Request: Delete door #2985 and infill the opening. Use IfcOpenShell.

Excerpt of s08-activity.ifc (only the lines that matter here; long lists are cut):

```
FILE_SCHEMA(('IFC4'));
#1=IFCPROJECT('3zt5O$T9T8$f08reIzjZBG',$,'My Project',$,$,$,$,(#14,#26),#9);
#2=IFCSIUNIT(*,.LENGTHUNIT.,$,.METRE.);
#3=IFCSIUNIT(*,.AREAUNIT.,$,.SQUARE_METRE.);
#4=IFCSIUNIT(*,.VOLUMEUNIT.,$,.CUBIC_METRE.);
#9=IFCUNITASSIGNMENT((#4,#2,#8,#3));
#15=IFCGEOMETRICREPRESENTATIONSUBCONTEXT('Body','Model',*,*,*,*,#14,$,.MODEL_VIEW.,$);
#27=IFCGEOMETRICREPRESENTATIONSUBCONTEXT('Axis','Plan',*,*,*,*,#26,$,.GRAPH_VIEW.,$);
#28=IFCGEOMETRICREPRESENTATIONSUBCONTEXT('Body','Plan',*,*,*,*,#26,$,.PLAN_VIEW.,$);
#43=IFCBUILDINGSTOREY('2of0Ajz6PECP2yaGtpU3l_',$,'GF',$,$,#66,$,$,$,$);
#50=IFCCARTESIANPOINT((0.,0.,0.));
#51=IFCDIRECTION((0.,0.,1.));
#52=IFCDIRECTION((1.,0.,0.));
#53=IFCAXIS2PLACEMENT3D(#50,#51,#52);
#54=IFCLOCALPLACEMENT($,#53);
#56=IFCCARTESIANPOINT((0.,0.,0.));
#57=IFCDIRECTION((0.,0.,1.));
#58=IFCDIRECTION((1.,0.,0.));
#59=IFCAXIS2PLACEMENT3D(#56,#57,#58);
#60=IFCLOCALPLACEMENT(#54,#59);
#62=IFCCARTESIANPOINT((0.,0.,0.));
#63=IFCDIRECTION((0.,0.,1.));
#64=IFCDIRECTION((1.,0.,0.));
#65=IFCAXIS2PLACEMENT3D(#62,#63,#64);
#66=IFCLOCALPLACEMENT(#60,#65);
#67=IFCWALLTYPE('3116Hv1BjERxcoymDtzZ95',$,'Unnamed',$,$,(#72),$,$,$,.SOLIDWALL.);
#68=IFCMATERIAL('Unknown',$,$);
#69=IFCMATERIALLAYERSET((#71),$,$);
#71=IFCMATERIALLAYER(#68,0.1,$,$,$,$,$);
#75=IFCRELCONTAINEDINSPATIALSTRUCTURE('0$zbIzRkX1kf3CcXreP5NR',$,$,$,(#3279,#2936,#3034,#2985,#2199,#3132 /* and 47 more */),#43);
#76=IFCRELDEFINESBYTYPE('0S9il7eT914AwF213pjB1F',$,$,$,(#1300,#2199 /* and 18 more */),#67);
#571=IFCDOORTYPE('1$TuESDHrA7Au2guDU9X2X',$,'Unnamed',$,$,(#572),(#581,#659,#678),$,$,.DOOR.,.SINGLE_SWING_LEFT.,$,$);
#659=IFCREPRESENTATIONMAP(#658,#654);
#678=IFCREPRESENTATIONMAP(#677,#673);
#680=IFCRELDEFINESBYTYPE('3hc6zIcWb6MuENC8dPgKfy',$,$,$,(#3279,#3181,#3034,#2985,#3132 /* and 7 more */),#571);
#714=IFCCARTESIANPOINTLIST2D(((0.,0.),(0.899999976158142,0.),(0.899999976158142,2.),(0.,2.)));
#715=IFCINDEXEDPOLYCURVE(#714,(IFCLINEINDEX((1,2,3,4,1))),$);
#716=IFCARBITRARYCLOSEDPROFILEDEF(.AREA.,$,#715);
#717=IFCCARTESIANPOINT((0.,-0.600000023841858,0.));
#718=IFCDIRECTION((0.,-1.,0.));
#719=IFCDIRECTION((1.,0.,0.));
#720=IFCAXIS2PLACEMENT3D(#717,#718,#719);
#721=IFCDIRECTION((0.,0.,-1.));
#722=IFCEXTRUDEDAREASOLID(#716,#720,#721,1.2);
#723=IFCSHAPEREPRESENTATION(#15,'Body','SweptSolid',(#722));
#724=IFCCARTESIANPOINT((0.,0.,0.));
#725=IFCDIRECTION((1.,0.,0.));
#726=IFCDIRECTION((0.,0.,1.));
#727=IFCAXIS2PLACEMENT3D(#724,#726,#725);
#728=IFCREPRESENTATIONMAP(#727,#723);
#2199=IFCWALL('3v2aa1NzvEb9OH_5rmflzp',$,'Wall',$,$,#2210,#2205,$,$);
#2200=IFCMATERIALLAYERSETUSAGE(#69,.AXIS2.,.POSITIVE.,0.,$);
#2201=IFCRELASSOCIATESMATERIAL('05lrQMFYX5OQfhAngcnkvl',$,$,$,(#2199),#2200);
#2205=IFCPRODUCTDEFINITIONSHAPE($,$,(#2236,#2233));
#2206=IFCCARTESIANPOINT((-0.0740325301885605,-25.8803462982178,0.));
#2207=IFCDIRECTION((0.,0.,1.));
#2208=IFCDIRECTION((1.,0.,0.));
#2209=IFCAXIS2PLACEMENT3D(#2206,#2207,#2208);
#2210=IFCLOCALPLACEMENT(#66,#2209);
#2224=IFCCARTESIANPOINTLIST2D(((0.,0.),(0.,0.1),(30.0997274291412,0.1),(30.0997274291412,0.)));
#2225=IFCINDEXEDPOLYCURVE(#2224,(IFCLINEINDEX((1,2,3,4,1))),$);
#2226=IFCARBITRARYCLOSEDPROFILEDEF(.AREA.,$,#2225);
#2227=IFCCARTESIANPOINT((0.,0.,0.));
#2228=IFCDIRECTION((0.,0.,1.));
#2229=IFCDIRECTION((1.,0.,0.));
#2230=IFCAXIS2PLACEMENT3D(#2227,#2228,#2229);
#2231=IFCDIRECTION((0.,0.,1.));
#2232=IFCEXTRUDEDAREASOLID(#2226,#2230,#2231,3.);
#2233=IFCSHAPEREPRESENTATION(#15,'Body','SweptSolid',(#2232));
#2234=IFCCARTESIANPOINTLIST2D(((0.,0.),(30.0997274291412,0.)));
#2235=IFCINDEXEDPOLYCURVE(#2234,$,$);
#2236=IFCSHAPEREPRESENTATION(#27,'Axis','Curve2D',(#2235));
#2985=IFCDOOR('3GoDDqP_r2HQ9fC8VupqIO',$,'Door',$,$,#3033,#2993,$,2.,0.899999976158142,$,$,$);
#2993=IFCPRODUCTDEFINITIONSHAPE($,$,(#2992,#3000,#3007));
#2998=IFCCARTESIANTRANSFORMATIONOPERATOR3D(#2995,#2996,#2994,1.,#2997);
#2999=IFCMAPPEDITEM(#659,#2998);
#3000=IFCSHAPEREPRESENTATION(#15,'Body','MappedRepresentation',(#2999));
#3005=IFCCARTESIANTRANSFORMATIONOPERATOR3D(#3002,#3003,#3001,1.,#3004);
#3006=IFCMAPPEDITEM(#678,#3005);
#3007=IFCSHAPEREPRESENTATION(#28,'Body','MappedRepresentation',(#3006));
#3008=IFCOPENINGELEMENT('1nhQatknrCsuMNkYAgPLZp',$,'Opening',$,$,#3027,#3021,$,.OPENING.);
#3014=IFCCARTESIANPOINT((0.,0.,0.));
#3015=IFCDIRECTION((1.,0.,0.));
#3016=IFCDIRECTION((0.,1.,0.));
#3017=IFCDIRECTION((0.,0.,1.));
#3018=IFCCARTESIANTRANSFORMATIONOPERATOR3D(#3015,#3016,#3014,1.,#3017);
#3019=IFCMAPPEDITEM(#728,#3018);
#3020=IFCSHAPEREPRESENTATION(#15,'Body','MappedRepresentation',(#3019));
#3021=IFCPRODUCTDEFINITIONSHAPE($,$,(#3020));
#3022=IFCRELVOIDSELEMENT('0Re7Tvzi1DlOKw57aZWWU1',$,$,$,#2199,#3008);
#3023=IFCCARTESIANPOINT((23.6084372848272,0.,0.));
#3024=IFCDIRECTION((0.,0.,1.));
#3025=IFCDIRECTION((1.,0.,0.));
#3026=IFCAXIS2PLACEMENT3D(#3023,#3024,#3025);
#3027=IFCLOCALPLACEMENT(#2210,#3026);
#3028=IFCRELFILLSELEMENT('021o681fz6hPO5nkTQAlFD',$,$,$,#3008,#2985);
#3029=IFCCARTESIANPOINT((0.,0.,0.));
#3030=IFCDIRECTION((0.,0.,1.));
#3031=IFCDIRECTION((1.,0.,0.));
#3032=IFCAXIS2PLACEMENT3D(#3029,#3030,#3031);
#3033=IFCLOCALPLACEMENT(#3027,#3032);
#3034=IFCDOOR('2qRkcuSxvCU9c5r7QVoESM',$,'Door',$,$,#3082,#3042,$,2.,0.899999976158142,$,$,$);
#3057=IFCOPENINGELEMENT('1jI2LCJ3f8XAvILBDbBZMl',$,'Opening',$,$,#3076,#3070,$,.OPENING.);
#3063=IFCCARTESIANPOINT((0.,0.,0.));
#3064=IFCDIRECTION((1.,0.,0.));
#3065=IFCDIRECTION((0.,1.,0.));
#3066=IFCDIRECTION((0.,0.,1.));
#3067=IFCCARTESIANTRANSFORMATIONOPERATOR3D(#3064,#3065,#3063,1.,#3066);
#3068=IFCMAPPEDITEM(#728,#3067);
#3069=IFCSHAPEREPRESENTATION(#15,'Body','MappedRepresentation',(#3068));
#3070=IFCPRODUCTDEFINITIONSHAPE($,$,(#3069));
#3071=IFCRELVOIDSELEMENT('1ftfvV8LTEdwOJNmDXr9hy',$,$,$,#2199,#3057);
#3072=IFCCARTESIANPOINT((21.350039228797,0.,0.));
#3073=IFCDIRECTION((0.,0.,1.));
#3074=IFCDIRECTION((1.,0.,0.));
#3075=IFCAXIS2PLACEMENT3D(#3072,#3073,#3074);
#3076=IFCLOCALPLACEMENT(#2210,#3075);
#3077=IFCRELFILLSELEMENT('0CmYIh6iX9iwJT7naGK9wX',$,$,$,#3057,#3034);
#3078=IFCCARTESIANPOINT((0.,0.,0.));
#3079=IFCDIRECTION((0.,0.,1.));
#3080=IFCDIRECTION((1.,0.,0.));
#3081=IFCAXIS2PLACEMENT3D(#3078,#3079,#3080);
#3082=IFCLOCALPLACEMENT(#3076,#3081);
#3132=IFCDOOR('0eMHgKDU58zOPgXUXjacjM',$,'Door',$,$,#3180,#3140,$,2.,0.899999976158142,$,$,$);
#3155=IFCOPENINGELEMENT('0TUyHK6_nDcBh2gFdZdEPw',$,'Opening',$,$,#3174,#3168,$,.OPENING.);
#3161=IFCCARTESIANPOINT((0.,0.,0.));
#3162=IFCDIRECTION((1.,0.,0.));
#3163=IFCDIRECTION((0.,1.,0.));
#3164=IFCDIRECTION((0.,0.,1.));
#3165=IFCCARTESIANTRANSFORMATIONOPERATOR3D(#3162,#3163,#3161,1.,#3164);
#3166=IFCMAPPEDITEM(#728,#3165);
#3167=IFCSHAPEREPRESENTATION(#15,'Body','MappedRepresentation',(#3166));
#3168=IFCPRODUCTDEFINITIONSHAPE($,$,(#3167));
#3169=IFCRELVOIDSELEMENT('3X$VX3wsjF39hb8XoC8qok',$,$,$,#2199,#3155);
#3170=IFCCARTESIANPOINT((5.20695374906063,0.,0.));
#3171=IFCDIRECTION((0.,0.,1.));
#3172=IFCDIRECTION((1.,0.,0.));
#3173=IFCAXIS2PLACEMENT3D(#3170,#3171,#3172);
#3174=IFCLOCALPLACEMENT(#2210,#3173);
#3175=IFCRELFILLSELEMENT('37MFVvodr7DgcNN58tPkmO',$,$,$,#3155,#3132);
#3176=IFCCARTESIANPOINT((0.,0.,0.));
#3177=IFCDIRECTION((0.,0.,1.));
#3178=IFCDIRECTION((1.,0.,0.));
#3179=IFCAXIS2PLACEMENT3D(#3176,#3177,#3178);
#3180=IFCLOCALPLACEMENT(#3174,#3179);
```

```python
import ifcopenshell
import ifcopenshell.api.feature
import ifcopenshell.api.root
import ifcopenshell.geom
import ifcopenshell.util.shape

model = ifcopenshell.open("s08-activity.ifc")
settings = ifcopenshell.geom.settings()


def volume(element):
    """Net volume in cubic metres, openings subtracted."""
    shape = ifcopenshell.geom.create_shape(settings, element)
    return ifcopenshell.util.shape.get_volume(shape.geometry)


door = model.by_guid("3GoDDqP_r2HQ9fC8VupqIO")
opening = door.FillsVoids[0].RelatingOpeningElement
wall = opening.VoidsElements[0].RelatingBuildingElement
before = volume(wall)

ifcopenshell.api.root.remove_product(model, product=door)
ifcopenshell.api.feature.remove_feature(model, feature=opening)

after = volume(wall)

print(f"wall volume {before:.3f} -> {after:.3f} m3")

model.write("s08-activity_edited.ifc")
```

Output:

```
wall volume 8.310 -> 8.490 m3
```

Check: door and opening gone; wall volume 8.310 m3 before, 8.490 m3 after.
